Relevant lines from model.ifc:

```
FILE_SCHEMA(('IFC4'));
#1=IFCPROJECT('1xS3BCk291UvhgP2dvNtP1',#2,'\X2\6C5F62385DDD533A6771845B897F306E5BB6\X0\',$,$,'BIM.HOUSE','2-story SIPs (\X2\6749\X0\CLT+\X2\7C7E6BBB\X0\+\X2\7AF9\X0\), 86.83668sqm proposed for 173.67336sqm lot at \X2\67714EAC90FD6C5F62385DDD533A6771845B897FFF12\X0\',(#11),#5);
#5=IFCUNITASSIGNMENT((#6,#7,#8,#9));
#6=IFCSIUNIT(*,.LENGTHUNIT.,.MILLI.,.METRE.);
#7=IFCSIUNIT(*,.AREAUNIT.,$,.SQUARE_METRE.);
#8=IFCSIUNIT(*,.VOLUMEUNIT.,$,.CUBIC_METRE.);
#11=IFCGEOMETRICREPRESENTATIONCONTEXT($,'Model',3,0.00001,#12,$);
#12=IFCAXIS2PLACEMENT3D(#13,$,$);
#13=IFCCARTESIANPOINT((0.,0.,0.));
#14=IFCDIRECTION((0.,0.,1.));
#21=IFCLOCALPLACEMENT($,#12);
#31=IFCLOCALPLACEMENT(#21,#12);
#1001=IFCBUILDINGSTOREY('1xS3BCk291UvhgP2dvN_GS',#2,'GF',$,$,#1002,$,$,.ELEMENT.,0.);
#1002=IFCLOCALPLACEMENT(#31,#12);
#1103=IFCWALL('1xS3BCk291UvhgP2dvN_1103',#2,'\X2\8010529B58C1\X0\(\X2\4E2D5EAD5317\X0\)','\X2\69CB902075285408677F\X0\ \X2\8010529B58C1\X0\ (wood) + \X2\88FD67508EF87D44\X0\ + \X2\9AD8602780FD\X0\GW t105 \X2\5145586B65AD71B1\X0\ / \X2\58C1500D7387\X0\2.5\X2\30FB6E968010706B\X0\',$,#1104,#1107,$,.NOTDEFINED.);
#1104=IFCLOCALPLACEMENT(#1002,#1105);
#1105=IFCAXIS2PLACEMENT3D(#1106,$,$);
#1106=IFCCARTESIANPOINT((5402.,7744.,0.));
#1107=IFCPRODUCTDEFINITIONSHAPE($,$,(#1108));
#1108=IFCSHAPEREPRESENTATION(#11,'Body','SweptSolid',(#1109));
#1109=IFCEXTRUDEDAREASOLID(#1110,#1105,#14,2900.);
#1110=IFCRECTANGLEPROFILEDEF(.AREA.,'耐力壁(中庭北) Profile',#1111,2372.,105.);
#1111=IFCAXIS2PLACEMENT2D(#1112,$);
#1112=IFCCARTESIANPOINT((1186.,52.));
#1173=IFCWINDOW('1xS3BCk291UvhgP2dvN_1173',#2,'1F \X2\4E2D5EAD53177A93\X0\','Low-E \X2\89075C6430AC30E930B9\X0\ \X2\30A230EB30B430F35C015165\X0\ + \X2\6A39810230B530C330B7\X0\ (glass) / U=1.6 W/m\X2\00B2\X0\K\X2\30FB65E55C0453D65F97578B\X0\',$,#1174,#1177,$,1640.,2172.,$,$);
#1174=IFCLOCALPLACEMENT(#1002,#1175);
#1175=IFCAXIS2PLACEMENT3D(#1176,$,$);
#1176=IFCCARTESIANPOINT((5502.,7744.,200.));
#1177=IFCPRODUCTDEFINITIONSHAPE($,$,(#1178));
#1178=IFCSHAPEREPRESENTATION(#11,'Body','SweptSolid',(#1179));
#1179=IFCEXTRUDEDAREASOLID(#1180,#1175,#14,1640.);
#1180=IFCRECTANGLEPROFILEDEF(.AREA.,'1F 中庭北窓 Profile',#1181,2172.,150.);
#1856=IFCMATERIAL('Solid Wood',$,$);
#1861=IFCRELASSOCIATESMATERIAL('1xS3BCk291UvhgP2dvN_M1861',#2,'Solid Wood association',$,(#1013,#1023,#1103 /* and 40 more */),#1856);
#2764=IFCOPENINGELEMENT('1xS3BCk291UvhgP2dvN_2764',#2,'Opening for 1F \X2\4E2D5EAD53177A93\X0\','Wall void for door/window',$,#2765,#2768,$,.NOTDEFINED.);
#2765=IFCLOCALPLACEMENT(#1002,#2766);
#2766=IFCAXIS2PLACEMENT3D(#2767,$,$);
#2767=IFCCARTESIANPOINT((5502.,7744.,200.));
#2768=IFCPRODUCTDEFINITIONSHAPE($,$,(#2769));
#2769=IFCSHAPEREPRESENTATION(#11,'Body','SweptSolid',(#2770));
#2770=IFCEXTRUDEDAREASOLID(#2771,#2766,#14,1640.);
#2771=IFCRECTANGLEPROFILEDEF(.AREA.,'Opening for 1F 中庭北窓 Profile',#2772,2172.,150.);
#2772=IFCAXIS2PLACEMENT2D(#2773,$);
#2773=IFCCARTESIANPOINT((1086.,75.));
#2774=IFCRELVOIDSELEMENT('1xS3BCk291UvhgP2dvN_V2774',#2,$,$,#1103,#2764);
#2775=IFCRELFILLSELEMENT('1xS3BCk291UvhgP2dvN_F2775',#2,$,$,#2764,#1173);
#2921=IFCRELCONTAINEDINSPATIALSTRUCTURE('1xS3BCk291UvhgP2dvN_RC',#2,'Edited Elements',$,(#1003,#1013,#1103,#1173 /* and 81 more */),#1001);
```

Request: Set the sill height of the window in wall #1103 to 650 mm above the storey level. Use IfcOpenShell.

```python
import numpy as np
import ifcopenshell
import ifcopenshell.api.geometry
import ifcopenshell.geom
import ifcopenshell.util.element
import ifcopenshell.util.placement
import ifcopenshell.util.shape
import ifcopenshell.util.unit

model = ifcopenshell.open("model.ifc")
unit_scale = ifcopenshell.util.unit.calculate_unit_scale(model)

window = model.by_id(1173)
opening = window.FillsVoids[0].RelatingOpeningElement
storey = ifcopenshell.util.element.get_container(window, ifc_class="IfcBuildingStorey")
level = ifcopenshell.util.placement.get_local_placement(storey.ObjectPlacement)[2, 3]

# The opening's origin need not be at the sill, so measure its lowest point.
shape = ifcopenshell.geom.create_shape(ifcopenshell.geom.settings(), opening)
bottom = ifcopenshell.util.shape.get_shape_bottom_elevation(shape, shape.geometry) / unit_scale
dz = level + 0.65 / unit_scale - bottom

shift = np.array([0.0, 0.0, dz])
# The window is not placed relative to its opening, so move both.
for product in (opening, window):
    matrix = ifcopenshell.util.placement.get_local_placement(product.ObjectPlacement)
    matrix[:3, 3] += shift
    ifcopenshell.api.geometry.edit_object_placement(model, product=product, matrix=matrix, is_si=False)

print(f"moved by {dz * unit_scale:+.3f} m")

model.write("model_updated.ifc")
```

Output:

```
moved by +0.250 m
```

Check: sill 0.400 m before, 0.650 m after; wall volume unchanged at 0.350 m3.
